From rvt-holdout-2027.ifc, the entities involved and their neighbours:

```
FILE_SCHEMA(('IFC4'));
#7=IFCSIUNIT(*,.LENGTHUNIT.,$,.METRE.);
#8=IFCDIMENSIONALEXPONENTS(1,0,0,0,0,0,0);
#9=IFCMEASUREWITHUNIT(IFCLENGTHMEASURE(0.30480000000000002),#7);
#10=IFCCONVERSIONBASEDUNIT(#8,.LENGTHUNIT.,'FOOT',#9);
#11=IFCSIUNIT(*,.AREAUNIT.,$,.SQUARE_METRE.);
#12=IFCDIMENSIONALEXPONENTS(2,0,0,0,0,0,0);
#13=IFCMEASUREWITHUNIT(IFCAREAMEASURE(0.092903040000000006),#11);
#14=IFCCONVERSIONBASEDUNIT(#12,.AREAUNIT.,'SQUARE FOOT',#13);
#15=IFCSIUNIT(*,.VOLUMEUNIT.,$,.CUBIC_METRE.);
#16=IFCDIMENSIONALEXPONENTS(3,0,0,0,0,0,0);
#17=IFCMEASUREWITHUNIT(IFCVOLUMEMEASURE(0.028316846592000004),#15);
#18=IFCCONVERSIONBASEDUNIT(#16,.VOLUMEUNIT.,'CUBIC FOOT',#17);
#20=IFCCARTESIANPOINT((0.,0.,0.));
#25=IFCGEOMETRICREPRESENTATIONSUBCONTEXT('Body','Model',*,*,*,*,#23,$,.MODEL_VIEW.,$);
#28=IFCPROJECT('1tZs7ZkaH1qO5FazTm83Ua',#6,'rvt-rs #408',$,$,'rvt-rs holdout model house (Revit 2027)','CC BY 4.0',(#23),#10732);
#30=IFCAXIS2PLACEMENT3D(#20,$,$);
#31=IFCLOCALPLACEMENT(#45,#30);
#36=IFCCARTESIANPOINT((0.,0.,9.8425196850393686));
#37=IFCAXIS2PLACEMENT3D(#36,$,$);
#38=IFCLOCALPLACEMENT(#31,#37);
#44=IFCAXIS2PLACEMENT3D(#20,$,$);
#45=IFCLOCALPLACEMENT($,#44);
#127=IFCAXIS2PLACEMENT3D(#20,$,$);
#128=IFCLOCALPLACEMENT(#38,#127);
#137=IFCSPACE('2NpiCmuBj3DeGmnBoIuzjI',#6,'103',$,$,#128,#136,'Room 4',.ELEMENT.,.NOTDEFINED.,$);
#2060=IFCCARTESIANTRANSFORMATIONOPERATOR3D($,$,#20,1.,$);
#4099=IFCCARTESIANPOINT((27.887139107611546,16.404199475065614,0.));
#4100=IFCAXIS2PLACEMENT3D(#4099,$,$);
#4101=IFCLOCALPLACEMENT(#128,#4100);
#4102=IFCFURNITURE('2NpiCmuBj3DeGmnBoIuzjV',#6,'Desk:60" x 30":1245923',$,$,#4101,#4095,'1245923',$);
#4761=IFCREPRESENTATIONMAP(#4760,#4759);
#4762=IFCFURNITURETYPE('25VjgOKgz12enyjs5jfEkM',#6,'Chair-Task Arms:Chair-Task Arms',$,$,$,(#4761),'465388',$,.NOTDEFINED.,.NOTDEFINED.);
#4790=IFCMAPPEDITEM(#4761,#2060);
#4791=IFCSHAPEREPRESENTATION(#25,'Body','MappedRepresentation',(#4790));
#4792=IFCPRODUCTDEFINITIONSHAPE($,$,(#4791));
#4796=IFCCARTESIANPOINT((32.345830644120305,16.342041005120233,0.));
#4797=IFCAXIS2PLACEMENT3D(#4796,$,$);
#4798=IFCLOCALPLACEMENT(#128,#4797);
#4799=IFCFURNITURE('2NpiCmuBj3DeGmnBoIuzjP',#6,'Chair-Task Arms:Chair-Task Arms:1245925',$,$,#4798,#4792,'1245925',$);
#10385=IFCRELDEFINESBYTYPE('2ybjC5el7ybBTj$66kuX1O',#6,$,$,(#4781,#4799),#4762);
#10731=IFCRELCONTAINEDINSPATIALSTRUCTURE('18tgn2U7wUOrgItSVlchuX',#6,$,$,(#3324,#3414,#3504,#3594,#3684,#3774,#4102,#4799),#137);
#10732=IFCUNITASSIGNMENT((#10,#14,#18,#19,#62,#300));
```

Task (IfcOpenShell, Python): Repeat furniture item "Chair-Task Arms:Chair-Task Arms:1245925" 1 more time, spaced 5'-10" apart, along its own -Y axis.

```python
import ifcopenshell
import ifcopenshell.api.geometry
import ifcopenshell.api.root
import ifcopenshell.util.element
import ifcopenshell.util.placement
import ifcopenshell.util.unit

model = ifcopenshell.open("rvt-holdout-2027.ifc")
unit_scale = ifcopenshell.util.unit.calculate_unit_scale(model)


def reuse_history(source, copy):
    """copy_class also copies each property set's owner history, people and application; keep the originals."""
    for rel in copy.IsDefinedBy:
        if rel.is_a("IfcRelDefinesByProperties") and (history := rel.RelatingPropertyDefinition.OwnerHistory):
            rel.RelatingPropertyDefinition.OwnerHistory = source.OwnerHistory
            ifcopenshell.util.element.remove_deep2(model, history)


source = model.by_guid("2NpiCmuBj3DeGmnBoIuzjP")
base = ifcopenshell.util.placement.get_local_placement(source.ObjectPlacement)
step = -base[:3, 1] * 70 * 0.0254 / unit_scale

for i in range(1, 2):
    copy = ifcopenshell.api.root.copy_class(model, product=source)
    copy.Representation = ifcopenshell.util.element.copy_deep(
        model, source.Representation, exclude=["IfcGeometricRepresentationContext", "IfcRepresentationMap"]
    )
    copy.Name = "Chair-Task Arms:Chair-Task Arms"
    copy.Tag = None
    reuse_history(source, copy)
    matrix = base.copy()
    matrix[:3, 3] += i * step
    print("added at", matrix[:3, 3].round(3) + 0.0)
    ifcopenshell.api.geometry.edit_object_placement(model, product=copy, matrix=matrix, is_si=False)

model.write("rvt-holdout-2027-out.ifc")
```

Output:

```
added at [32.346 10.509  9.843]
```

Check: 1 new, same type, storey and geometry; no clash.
